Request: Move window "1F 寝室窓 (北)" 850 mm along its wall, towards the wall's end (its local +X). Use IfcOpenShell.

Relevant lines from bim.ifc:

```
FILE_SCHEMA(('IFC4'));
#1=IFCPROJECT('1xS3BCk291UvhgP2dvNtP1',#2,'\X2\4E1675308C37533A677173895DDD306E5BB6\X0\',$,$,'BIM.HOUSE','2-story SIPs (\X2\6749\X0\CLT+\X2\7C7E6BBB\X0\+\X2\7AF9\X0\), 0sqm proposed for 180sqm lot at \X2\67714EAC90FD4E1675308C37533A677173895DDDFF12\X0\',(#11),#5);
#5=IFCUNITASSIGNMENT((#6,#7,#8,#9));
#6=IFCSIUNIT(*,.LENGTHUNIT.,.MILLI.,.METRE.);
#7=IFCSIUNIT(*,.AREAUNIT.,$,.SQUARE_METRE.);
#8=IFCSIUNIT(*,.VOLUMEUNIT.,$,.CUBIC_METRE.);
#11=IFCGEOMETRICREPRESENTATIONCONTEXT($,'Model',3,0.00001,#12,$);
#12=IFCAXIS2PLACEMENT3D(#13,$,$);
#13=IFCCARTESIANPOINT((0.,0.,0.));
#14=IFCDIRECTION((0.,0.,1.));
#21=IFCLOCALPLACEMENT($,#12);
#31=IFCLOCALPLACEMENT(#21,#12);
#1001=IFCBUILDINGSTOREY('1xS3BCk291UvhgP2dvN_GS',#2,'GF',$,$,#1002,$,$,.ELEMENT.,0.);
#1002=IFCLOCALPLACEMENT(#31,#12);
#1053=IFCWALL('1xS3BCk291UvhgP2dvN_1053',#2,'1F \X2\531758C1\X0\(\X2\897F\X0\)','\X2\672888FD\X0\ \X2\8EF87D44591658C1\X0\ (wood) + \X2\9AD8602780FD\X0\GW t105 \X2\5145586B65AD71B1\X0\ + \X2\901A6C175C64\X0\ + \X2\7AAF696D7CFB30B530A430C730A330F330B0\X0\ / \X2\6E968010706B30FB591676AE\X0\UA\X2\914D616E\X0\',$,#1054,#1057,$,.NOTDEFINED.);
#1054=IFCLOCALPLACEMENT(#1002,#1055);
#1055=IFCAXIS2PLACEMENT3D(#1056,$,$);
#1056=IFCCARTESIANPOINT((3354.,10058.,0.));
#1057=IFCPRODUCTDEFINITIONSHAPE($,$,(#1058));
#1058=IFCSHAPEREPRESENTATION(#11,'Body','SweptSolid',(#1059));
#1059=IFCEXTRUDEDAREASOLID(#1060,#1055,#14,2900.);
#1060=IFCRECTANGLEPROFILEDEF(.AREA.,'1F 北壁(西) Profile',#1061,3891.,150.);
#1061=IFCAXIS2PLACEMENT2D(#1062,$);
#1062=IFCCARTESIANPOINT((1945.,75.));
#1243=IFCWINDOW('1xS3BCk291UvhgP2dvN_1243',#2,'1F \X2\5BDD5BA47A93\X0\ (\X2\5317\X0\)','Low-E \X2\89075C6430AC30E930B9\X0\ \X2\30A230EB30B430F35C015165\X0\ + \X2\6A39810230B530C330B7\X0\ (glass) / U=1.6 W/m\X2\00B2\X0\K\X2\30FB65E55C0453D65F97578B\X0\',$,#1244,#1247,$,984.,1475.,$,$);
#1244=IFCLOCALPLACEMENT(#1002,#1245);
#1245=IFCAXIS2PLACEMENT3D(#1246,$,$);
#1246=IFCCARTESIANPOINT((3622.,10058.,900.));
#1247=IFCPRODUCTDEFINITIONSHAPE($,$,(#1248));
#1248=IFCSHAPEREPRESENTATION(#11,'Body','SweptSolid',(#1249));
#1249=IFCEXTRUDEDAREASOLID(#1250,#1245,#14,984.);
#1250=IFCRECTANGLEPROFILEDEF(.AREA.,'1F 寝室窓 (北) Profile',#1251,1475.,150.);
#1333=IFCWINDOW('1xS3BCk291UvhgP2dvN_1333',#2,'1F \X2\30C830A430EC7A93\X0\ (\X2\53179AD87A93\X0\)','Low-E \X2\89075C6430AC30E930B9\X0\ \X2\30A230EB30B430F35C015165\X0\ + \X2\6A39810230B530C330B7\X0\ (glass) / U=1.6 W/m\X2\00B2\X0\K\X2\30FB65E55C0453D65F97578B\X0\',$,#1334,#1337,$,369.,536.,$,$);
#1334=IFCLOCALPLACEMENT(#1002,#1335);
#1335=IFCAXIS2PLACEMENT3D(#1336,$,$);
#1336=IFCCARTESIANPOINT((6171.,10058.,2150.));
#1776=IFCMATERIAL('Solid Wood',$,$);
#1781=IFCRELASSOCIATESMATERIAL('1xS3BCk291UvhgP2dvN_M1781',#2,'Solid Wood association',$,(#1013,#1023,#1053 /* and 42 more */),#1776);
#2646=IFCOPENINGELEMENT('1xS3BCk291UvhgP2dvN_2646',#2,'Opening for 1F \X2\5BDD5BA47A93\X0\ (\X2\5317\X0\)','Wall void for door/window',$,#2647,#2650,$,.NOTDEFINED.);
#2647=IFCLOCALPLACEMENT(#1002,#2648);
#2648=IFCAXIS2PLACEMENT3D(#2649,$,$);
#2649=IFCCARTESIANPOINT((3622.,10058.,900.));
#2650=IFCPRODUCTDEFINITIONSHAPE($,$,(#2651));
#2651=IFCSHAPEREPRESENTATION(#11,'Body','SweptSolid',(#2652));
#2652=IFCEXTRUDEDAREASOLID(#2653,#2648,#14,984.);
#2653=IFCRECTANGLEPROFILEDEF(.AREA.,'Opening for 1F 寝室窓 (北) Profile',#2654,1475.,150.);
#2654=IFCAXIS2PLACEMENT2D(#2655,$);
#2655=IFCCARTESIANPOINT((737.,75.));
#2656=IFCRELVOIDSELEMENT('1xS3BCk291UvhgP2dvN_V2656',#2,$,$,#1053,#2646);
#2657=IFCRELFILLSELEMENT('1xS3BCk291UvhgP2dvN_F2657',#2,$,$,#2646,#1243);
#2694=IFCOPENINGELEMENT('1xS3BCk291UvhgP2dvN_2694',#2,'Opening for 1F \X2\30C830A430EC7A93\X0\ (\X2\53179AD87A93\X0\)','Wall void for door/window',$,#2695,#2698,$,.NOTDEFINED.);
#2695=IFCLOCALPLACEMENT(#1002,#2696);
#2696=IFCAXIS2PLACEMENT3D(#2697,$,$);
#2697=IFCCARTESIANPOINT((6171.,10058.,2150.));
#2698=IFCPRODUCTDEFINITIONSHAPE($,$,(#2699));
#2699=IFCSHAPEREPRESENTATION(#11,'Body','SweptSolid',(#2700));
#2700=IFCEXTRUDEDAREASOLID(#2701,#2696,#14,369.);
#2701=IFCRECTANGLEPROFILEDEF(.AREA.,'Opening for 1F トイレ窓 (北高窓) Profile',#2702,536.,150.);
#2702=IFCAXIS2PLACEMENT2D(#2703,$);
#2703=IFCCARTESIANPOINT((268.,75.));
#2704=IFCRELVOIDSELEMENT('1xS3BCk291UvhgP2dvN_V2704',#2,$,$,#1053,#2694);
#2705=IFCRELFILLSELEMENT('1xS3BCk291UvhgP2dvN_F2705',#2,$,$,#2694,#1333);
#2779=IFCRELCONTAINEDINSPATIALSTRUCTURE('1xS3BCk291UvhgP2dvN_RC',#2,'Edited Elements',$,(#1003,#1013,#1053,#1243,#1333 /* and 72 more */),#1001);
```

```python
import ifcopenshell
import ifcopenshell.api.geometry
import ifcopenshell.util.placement

model = ifcopenshell.open("bim.ifc")

window = model.by_id(1243)
opening = window.FillsVoids[0].RelatingOpeningElement
wall = opening.VoidsElements[0].RelatingBuildingElement

wall_matrix = ifcopenshell.util.placement.get_local_placement(wall.ObjectPlacement)
shift = wall_matrix[:3, 0] * 850.0
before = ifcopenshell.util.placement.get_local_placement(window.ObjectPlacement)[:3, 3].copy()

# The window is not placed relative to its opening, so move both.
for product in (opening, window):
    matrix = ifcopenshell.util.placement.get_local_placement(product.ObjectPlacement)
    matrix[:3, 3] += shift
    ifcopenshell.api.geometry.edit_object_placement(model, product=product, matrix=matrix, is_si=False)

after = ifcopenshell.util.placement.get_local_placement(window.ObjectPlacement)[:3, 3]
print("window moved by", (after - before).round(3) + 0.0)

model.write("bim_v2.ifc")
```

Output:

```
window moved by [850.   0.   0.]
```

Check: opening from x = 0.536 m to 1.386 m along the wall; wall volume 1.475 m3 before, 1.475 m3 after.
